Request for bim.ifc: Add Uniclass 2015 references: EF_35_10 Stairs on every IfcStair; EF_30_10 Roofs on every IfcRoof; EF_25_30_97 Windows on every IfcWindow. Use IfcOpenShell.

First a look at what the model holds.

```python
import ifcopenshell

model = ifcopenshell.open("bim.ifc")
print(model.schema)
print("classifications:", [c.Name for c in model.by_type("IfcClassification")])
for ifc_class in ("IfcDoor", "IfcRoof", "IfcStair", "IfcWall", "IfcWindow"):
    print(ifc_class, len(model.by_type(ifc_class)))
```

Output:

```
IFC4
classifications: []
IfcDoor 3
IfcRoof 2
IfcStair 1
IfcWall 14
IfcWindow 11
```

```python
import ifcopenshell
import ifcopenshell.api.classification

model = ifcopenshell.open("bim.ifc")

system = ifcopenshell.api.classification.add_classification(model, classification="Uniclass 2015")

codes = {
    "IfcStair": ("EF_35_10", "Stairs"),
    "IfcRoof": ("EF_30_10", "Roofs"),
    "IfcWindow": ("EF_25_30_97", "Windows"),
}
for ifc_class, (code, name) in codes.items():
    products = model.by_type(ifc_class)
    ifcopenshell.api.classification.add_reference(
        model, products=products, classification=system, identification=code, name=name
    )
    print(code, len(products))

model.write("bim_updated.ifc")
```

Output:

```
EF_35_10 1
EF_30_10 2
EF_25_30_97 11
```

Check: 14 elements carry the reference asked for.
